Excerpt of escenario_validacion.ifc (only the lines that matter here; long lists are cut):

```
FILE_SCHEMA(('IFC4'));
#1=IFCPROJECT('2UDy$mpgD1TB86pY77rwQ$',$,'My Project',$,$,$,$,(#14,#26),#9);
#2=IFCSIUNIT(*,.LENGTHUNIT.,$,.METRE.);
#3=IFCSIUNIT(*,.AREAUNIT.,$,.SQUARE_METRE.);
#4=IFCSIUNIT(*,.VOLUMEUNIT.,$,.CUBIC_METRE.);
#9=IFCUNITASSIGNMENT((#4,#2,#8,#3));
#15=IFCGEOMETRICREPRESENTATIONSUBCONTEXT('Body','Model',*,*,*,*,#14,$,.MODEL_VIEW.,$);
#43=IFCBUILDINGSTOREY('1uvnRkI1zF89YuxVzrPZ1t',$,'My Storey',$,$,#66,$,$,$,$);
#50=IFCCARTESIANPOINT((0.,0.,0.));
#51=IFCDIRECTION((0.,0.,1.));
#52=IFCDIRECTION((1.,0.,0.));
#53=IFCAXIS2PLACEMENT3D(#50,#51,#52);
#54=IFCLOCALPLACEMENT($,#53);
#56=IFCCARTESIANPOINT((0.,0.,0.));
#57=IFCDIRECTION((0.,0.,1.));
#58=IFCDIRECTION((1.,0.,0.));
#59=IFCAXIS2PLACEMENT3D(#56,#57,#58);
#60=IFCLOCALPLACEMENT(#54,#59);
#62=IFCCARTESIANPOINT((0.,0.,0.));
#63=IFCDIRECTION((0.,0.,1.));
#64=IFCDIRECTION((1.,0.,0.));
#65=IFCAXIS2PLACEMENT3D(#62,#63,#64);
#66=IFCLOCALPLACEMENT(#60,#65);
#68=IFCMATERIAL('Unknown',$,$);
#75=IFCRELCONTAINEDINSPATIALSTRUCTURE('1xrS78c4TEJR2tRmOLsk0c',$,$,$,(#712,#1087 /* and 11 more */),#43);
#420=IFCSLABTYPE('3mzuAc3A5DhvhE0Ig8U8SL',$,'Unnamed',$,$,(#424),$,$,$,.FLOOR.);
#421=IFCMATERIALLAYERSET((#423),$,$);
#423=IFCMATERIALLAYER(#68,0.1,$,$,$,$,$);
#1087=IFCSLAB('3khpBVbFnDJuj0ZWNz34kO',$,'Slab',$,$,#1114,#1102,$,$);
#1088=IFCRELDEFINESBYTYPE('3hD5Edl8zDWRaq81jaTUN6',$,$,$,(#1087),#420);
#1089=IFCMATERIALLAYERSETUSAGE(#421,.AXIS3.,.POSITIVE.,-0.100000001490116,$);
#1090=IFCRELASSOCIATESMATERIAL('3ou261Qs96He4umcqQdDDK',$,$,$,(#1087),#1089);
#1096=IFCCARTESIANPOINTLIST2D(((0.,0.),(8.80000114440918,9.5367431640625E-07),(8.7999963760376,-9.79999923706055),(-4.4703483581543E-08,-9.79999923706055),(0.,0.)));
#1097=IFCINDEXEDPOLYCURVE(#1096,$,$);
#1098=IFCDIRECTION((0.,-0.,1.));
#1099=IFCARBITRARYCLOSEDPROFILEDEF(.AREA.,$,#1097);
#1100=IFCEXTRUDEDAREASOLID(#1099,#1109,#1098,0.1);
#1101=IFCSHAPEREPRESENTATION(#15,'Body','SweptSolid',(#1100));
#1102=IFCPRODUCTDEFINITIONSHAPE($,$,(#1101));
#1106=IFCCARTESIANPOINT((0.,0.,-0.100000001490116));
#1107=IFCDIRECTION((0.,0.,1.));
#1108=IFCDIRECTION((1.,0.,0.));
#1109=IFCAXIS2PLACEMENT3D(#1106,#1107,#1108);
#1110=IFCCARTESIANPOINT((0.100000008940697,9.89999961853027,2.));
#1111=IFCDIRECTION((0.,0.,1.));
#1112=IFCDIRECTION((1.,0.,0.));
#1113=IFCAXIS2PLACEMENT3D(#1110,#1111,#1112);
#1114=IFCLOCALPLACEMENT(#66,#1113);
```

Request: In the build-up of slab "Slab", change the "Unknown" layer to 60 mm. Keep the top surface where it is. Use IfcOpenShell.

```python
import ifcopenshell
import ifcopenshell.util.element
import ifcopenshell.util.representation
import ifcopenshell.util.unit

model = ifcopenshell.open("escenario_validacion.ifc")
unit_scale = ifcopenshell.util.unit.calculate_unit_scale(model)

layer_set = model.by_id(421)
layer = next(l for l in layer_set.MaterialLayers if l.Material and l.Material.Name == "Unknown")
change = 0.06 / unit_scale - layer.LayerThickness
layer.LayerThickness += change

# Geometry does not follow the layer set by itself.
slabs = [e for e in ifcopenshell.util.element.get_elements_by_material(model, layer_set) if e.is_a("IfcSlab")]
for slab in sorted(slabs, key=lambda e: e.id()):
    body = ifcopenshell.util.representation.get_representation(slab, "Model", "Body")
    solid = body.Items[0]
    old_depth = solid.Depth
    solid.Depth += change
    # Extruded upwards: lower the start of the extrusion so the top stays.
    x, y, z = solid.Position.Location.Coordinates
    solid.Position.Location = model.createIfcCartesianPoint((x, y, z - change))
    print(slab.id(), f"{old_depth:g} -> {solid.Depth:g}")

# The layers are counted up from the underside, which has moved.
for usage in {ifcopenshell.util.element.get_material(slab) for slab in slabs}:
    usage.OffsetFromReferenceLine -= change

model.write("escenario_validacion_edited.ifc")
```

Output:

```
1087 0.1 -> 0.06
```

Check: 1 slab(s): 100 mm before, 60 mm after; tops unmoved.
